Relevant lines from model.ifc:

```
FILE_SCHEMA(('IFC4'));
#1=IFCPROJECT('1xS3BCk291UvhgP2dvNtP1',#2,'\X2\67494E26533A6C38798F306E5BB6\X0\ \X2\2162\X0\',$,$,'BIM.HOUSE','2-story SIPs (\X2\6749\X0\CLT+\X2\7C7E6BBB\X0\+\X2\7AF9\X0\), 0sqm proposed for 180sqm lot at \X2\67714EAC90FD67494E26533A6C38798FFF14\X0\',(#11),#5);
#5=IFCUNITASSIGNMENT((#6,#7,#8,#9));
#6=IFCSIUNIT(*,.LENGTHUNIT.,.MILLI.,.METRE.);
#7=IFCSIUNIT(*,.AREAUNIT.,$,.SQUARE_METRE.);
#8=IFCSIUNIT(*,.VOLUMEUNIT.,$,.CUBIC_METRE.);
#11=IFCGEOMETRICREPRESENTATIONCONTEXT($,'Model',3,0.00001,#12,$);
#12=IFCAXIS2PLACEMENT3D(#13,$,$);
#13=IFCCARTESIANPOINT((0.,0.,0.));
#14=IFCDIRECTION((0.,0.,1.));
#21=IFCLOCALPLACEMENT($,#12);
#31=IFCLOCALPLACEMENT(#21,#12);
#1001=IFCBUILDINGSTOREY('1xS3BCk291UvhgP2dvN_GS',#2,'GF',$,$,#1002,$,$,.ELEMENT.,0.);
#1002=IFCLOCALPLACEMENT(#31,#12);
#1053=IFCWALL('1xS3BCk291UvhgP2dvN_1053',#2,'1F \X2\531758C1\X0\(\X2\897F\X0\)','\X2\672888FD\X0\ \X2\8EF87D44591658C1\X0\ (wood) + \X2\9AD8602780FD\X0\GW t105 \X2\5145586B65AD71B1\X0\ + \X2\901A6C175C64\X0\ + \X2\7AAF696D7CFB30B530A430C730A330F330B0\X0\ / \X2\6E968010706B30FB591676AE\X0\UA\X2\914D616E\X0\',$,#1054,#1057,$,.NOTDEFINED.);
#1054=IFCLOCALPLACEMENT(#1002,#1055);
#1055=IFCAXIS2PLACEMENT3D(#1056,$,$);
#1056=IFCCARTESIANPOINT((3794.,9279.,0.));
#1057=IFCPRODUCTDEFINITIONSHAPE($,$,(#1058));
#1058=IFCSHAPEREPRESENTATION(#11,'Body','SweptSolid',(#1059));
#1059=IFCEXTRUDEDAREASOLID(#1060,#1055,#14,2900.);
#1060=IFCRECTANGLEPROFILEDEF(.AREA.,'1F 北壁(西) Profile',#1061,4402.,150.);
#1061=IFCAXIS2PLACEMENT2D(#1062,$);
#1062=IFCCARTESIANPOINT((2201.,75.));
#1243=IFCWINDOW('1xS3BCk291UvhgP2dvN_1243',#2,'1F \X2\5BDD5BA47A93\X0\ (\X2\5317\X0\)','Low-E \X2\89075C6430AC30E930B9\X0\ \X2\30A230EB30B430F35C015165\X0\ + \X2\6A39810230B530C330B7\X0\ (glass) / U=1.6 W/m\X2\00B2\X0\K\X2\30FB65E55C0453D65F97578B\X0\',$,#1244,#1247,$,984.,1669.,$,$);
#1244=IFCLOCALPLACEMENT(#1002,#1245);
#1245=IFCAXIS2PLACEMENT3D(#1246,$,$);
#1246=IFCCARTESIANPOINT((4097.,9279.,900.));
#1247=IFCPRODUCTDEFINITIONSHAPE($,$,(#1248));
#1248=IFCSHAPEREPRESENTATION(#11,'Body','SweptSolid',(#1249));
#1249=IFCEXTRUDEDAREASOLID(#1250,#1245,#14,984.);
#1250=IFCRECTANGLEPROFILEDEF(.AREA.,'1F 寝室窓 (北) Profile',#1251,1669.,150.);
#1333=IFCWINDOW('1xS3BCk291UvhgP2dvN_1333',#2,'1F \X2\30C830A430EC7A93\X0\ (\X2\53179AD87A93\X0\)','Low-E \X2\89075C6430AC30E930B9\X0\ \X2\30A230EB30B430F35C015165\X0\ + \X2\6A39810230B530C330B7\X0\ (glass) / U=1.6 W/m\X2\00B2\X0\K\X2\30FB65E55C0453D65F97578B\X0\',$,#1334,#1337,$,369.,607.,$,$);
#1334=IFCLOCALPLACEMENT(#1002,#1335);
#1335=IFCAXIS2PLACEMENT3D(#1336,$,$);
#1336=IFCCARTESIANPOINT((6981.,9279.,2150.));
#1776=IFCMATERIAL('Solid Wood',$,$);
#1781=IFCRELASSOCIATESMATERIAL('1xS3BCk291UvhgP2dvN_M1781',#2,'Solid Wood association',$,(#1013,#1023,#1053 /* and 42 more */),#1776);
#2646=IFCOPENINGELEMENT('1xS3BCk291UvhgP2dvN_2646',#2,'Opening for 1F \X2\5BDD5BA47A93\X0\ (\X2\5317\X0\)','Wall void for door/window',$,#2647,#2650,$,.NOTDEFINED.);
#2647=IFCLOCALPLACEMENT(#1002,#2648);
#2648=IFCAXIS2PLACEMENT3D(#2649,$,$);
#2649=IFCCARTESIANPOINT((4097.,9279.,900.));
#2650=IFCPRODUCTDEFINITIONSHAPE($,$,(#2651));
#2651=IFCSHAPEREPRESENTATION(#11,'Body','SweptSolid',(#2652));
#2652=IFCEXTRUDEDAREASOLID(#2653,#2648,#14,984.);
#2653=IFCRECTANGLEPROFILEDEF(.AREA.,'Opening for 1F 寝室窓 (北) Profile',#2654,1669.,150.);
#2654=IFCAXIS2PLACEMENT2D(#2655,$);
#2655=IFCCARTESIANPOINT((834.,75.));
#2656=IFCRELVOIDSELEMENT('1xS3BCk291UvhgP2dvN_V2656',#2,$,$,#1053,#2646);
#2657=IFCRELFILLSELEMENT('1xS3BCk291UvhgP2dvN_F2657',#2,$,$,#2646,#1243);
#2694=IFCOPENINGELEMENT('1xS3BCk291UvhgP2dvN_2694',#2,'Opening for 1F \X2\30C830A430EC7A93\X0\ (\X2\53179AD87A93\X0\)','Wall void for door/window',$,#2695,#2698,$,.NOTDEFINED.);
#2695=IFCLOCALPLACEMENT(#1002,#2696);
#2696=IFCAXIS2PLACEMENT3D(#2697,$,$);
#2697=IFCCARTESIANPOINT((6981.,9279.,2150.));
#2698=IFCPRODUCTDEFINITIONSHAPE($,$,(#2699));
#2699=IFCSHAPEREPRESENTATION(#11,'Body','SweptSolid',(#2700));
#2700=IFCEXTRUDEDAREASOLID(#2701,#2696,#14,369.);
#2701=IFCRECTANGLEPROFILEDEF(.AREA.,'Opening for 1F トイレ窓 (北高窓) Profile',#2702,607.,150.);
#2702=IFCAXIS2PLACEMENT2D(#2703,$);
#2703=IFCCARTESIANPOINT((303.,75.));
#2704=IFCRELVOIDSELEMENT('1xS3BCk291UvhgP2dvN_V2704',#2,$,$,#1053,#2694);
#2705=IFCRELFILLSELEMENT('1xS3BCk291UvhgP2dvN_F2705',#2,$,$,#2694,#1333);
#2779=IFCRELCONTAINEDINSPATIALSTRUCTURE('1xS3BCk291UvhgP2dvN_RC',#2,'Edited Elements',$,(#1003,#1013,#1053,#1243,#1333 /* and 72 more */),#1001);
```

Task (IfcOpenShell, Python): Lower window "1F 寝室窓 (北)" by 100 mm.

```python
import numpy as np
import ifcopenshell
import ifcopenshell.api.geometry
import ifcopenshell.util.placement
import ifcopenshell.util.unit

model = ifcopenshell.open("model.ifc")
unit_scale = ifcopenshell.util.unit.calculate_unit_scale(model)

window = model.by_guid("1xS3BCk291UvhgP2dvN_1243")
opening = window.FillsVoids[0].RelatingOpeningElement
dz = -0.1 / unit_scale

shift = np.array([0.0, 0.0, dz])
# The window is not placed relative to its opening, so move both.
for product in (opening, window):
    matrix = ifcopenshell.util.placement.get_local_placement(product.ObjectPlacement)
    matrix[:3, 3] += shift
    ifcopenshell.api.geometry.edit_object_placement(model, product=product, matrix=matrix, is_si=False)

print(f"moved by {dz * unit_scale:+.3f} m")

model.write("model_updated.ifc")
```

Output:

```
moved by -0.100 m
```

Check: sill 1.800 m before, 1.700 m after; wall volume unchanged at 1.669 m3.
